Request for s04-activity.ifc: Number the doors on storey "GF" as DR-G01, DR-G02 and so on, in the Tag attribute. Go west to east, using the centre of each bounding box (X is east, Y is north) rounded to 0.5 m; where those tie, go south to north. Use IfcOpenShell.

First a look at what the model holds.

```python
import ifcopenshell
import ifcopenshell.util.element
import ifcopenshell.util.placement

model = ifcopenshell.open("s04-activity.ifc")
print(model.schema)
storey = next(s for s in model.by_type("IfcBuildingStorey") if s.Name == "GF")
doors = [e for e in ifcopenshell.util.element.get_decomposition(storey) if e.is_a("IfcDoor")]
for e in sorted(doors, key=lambda e: e.id()):
    origin = ifcopenshell.util.placement.get_local_placement(e.ObjectPlacement)[:3, 3]
    print(e.id(), e.Tag, e.Name, origin.round(2) + 0.0, sep=" | ")
```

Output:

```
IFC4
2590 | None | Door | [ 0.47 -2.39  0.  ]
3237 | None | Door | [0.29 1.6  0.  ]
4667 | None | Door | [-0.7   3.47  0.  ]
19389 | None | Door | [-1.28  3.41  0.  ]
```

```python
import ifcopenshell
import ifcopenshell.geom
import ifcopenshell.util.element
import ifcopenshell.util.shape

model = ifcopenshell.open("s04-activity.ifc")
settings = ifcopenshell.geom.settings()
settings.set("use-world-coords", True)


def centre(element):
    shape = ifcopenshell.geom.create_shape(settings, element)
    return ifcopenshell.util.shape.get_bbox_centroid(shape.geometry)


storey = next(s for s in model.by_type("IfcBuildingStorey") if s.Name == "GF")
doors = [e for e in ifcopenshell.util.element.get_decomposition(storey) if e.is_a("IfcDoor")]

# Insertion points can sit at a corner or the storey origin, so sort by the geometry (in metres).
centres = {e: centre(e) for e in doors}
doors.sort(key=lambda e: (round(centres[e][0] / 0.5), centres[e][1]))

for i, e in enumerate(doors, start=1):
    number = f"DR-G{i:02d}"
    e.Tag = number
    print(e.id(), number)

model.write("s04-activity_updated.ifc")
```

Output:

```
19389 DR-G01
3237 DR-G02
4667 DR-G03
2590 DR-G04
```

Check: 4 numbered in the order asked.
